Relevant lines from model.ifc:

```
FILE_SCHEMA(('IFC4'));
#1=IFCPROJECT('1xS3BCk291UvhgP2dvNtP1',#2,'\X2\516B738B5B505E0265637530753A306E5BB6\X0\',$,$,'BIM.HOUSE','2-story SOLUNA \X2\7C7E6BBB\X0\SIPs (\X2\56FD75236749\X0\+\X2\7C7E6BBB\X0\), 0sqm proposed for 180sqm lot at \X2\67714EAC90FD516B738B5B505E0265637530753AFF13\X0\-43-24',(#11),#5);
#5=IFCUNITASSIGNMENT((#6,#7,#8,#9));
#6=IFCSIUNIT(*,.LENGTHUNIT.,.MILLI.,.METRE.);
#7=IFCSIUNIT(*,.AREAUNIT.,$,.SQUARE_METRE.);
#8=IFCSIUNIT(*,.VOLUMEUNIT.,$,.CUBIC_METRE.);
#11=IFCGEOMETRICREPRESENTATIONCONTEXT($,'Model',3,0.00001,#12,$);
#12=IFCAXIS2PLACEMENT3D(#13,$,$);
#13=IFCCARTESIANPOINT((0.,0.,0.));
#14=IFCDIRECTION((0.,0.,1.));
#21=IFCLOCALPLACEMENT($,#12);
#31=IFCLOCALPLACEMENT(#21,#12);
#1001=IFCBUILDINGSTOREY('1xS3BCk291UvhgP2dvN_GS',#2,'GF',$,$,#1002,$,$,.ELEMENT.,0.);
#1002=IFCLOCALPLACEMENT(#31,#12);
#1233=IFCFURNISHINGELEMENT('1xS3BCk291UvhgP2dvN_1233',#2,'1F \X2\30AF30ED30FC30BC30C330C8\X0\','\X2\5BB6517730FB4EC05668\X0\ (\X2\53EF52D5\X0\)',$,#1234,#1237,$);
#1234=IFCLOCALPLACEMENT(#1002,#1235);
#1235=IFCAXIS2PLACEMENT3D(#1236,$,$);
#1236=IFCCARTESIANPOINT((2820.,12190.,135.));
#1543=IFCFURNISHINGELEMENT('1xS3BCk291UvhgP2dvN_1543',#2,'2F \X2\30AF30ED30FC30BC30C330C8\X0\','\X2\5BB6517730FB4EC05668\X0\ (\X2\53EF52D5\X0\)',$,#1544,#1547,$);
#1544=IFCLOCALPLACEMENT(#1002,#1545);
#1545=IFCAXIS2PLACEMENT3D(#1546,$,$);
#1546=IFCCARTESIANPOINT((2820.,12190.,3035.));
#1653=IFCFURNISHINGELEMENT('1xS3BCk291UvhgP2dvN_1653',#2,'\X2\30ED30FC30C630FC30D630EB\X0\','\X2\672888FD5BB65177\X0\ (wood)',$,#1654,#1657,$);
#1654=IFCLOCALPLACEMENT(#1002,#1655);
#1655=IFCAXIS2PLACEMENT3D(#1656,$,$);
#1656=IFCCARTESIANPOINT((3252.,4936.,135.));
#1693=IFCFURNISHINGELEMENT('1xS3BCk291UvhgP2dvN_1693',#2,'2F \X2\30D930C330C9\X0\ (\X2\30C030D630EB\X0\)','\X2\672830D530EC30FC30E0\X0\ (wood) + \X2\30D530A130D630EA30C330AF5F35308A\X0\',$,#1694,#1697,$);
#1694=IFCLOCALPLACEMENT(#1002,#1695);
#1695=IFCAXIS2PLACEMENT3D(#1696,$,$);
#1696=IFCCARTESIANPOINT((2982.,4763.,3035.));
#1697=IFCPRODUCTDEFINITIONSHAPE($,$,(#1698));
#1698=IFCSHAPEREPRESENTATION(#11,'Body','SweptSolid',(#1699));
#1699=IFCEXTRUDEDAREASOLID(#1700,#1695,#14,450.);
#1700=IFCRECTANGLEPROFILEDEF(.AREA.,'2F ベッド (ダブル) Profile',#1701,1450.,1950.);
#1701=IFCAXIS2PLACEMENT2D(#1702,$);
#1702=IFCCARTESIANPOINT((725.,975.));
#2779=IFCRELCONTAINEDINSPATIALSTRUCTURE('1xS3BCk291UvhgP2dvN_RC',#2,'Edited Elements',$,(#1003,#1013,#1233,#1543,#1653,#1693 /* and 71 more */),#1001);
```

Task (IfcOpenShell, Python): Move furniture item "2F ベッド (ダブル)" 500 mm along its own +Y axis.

```python
import ifcopenshell
import ifcopenshell.api.geometry
import ifcopenshell.util.placement

model = ifcopenshell.open("model.ifc")

item = model.by_id(1693)
matrix = ifcopenshell.util.placement.get_local_placement(item.ObjectPlacement)
matrix[:3, 3] += matrix[:3, 1] * 500.0
ifcopenshell.api.geometry.edit_object_placement(model, product=item, matrix=matrix, is_si=False)

print(ifcopenshell.util.placement.get_local_placement(item.ObjectPlacement).round(3) + 0.0)

model.write("model-out.ifc")
```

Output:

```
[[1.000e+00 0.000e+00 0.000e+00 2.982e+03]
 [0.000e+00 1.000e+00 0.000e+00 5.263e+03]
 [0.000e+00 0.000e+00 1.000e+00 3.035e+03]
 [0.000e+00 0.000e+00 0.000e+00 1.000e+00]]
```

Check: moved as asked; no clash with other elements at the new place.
